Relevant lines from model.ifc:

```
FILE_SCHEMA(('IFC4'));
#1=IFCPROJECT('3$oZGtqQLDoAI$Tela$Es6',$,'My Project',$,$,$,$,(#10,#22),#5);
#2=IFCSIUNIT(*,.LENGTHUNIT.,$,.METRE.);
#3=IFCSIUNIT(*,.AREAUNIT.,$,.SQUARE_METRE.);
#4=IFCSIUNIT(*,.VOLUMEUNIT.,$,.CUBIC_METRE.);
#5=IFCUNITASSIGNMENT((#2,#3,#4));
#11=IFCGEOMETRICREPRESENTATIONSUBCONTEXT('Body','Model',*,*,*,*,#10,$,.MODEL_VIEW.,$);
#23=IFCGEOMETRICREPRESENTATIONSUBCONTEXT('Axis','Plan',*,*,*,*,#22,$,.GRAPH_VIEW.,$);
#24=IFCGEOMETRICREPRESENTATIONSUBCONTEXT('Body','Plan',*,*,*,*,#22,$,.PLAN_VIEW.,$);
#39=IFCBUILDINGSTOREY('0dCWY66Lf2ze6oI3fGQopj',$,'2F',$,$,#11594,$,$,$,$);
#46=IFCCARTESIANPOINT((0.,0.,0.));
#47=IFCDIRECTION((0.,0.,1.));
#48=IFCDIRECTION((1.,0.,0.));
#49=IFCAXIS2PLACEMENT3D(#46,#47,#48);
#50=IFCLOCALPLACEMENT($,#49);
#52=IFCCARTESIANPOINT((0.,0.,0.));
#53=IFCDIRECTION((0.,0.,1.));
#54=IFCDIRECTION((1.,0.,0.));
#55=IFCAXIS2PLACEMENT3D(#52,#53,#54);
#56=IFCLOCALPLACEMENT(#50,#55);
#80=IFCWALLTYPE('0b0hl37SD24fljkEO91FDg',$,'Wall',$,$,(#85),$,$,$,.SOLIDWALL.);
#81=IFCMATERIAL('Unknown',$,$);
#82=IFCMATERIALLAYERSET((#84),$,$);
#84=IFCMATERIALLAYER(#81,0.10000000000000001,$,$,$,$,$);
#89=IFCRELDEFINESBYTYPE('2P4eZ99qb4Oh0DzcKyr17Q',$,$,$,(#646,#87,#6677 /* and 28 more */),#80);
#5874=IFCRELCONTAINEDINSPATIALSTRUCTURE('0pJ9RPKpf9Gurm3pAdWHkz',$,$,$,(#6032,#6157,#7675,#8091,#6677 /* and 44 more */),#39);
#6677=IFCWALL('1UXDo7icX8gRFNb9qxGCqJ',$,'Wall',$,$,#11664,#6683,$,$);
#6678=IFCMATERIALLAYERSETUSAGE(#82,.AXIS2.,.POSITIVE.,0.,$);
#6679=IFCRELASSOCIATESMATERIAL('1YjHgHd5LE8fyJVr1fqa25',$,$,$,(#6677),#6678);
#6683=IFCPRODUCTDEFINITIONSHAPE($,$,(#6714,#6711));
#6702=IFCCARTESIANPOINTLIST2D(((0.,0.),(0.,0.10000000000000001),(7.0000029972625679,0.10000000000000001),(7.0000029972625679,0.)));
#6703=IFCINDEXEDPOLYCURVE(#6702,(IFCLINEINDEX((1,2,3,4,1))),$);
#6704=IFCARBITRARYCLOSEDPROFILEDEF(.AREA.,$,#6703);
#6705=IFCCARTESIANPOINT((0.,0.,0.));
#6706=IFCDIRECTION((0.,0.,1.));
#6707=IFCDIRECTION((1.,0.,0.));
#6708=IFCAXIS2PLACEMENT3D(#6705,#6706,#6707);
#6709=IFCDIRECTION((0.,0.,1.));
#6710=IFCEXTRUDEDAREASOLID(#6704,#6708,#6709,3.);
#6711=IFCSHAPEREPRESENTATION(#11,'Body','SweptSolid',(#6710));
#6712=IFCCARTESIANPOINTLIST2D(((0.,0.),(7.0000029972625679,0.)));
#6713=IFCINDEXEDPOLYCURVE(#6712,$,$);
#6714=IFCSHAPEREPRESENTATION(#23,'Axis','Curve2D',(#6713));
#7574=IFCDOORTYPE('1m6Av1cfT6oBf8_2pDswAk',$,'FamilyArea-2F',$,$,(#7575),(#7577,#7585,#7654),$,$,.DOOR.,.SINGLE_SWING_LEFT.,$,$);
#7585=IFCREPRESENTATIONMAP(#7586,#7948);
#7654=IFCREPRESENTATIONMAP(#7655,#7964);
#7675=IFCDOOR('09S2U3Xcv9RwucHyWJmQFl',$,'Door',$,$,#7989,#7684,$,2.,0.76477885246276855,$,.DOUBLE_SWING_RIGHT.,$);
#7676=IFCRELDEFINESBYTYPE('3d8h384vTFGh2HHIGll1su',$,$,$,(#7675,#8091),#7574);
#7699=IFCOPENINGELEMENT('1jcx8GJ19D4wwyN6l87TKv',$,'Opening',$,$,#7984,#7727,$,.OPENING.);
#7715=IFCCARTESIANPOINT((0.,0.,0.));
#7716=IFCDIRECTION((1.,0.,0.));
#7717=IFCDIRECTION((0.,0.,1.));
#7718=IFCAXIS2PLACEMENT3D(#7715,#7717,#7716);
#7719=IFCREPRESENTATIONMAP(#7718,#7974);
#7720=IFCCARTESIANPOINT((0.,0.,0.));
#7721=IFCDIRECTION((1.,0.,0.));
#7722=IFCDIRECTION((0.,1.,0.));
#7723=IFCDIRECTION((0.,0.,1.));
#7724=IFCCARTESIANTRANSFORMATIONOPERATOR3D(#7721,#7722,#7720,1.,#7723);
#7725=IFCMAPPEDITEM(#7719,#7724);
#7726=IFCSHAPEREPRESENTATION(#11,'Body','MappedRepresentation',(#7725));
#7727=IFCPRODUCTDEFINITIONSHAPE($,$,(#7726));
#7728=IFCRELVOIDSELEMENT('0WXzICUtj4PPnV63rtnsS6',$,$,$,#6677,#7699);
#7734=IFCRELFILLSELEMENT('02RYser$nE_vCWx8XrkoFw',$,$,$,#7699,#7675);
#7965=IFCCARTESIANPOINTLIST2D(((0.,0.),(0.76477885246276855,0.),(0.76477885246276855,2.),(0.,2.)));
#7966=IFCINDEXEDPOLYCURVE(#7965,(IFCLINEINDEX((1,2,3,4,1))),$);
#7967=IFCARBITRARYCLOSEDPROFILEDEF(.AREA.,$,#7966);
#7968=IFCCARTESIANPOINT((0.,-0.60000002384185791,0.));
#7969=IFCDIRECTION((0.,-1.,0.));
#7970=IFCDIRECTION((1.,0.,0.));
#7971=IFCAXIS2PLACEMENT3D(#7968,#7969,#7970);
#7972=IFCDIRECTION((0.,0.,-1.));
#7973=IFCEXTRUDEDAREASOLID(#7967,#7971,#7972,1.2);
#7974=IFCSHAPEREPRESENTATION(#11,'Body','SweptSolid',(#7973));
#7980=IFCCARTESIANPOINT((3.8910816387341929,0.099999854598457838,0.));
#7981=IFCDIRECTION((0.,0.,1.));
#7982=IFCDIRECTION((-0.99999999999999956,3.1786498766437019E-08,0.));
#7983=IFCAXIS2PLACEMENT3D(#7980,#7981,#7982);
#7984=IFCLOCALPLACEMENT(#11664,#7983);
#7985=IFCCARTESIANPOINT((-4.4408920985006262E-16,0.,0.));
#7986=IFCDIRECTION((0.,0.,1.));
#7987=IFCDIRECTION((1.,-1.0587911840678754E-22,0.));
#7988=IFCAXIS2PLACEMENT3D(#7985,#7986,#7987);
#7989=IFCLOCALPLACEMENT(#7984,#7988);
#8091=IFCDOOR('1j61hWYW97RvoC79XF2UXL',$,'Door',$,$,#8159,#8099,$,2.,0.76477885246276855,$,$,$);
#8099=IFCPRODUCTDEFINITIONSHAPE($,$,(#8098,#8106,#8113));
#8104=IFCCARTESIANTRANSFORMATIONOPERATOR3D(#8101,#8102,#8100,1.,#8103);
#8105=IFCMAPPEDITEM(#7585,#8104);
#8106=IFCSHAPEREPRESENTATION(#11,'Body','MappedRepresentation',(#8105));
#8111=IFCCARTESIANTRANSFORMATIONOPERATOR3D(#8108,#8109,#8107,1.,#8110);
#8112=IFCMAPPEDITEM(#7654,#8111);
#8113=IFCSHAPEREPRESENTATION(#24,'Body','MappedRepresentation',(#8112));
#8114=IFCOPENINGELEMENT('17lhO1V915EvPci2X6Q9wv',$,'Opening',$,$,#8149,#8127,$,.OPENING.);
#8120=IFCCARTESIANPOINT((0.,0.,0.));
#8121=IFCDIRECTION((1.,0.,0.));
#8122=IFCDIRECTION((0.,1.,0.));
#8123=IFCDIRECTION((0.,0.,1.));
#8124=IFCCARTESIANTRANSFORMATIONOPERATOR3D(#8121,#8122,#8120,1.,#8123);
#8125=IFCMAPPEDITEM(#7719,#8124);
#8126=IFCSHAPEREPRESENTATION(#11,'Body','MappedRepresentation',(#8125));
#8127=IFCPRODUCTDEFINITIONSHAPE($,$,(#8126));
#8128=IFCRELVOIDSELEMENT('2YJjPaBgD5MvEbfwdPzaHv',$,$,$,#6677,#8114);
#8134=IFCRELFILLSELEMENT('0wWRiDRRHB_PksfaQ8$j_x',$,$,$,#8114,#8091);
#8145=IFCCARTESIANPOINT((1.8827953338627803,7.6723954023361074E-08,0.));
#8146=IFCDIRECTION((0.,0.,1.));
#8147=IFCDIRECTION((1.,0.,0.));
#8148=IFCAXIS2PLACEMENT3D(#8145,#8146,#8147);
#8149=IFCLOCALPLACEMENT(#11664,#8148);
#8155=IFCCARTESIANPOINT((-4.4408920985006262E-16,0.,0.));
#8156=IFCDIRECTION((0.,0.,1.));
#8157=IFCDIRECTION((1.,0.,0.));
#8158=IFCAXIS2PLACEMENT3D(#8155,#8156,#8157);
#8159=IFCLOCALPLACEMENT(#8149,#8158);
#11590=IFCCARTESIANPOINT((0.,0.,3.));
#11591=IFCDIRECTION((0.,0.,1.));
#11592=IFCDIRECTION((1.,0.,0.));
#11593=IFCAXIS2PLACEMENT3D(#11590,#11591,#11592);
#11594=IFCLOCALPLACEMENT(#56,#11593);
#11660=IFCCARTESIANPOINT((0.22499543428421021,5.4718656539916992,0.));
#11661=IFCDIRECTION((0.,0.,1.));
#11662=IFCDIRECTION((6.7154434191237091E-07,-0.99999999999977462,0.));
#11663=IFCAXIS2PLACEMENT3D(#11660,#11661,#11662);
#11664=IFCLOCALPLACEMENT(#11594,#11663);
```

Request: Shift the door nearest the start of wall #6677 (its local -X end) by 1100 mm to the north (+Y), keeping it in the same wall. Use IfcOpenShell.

```python
import ifcopenshell
import ifcopenshell.api.geometry
import ifcopenshell.util.placement
import ifcopenshell.util.unit

model = ifcopenshell.open("model.ifc")
unit_scale = ifcopenshell.util.unit.calculate_unit_scale(model)

door = model.by_id(8091)
opening = door.FillsVoids[0].RelatingOpeningElement
wall = opening.VoidsElements[0].RelatingBuildingElement

wall_matrix = ifcopenshell.util.placement.get_local_placement(wall.ObjectPlacement)
shift = wall_matrix[:3, 0] * -1.1 / unit_scale
before = ifcopenshell.util.placement.get_local_placement(door.ObjectPlacement)[:3, 3].copy()

# The door is placed relative to its opening, so it follows when the opening moves.
matrix = ifcopenshell.util.placement.get_local_placement(opening.ObjectPlacement)
matrix[:3, 3] += shift
ifcopenshell.api.geometry.edit_object_placement(
    model, product=opening, matrix=matrix, is_si=False, should_transform_children=True
)

after = ifcopenshell.util.placement.get_local_placement(door.ObjectPlacement)[:3, 3]
print("door moved by", (after - before).round(3) + 0.0)

model.write("model_edited.ifc")
```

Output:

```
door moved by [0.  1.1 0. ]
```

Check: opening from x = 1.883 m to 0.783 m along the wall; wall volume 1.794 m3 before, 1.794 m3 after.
